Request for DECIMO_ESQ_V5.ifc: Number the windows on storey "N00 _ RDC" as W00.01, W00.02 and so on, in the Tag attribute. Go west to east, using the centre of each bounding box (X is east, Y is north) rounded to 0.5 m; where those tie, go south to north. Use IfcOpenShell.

First a look at what the model holds.

```python
import ifcopenshell
import ifcopenshell.util.element
import ifcopenshell.util.placement

model = ifcopenshell.open("DECIMO_ESQ_V5.ifc")
print(model.schema)
storey = next(s for s in model.by_type("IfcBuildingStorey") if s.Name == "N00 _ RDC")
windows = [e for e in ifcopenshell.util.element.get_decomposition(storey) if e.is_a("IfcWindow")]
for e in sorted(windows, key=lambda e: e.id()):
    origin = ifcopenshell.util.placement.get_local_placement(e.ObjectPlacement)[:3, 3]
    print(e.id(), e.Tag, e.Name, origin.round(2) + 0.0, sep=" | ")
```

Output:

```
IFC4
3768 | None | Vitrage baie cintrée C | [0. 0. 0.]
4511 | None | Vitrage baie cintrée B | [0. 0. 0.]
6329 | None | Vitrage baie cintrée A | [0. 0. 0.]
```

```python
import ifcopenshell
import ifcopenshell.geom
import ifcopenshell.util.element
import ifcopenshell.util.shape

model = ifcopenshell.open("DECIMO_ESQ_V5.ifc")
settings = ifcopenshell.geom.settings()
settings.set("use-world-coords", True)


def centre(element):
    shape = ifcopenshell.geom.create_shape(settings, element)
    return ifcopenshell.util.shape.get_bbox_centroid(shape.geometry)


storey = next(s for s in model.by_type("IfcBuildingStorey") if s.Name == "N00 _ RDC")
windows = [e for e in ifcopenshell.util.element.get_decomposition(storey) if e.is_a("IfcWindow")]

# Insertion points can sit at a corner or the storey origin, so sort by the geometry (in metres).
centres = {e: centre(e) for e in windows}
windows.sort(key=lambda e: (round(centres[e][0] / 0.5), centres[e][1]))

for i, e in enumerate(windows, start=1):
    number = f"W00.{i:02d}"
    e.Tag = number
    print(e.id(), number)

model.write("DECIMO_ESQ_V5_v2.ifc")
```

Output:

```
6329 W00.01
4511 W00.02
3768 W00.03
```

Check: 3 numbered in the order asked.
